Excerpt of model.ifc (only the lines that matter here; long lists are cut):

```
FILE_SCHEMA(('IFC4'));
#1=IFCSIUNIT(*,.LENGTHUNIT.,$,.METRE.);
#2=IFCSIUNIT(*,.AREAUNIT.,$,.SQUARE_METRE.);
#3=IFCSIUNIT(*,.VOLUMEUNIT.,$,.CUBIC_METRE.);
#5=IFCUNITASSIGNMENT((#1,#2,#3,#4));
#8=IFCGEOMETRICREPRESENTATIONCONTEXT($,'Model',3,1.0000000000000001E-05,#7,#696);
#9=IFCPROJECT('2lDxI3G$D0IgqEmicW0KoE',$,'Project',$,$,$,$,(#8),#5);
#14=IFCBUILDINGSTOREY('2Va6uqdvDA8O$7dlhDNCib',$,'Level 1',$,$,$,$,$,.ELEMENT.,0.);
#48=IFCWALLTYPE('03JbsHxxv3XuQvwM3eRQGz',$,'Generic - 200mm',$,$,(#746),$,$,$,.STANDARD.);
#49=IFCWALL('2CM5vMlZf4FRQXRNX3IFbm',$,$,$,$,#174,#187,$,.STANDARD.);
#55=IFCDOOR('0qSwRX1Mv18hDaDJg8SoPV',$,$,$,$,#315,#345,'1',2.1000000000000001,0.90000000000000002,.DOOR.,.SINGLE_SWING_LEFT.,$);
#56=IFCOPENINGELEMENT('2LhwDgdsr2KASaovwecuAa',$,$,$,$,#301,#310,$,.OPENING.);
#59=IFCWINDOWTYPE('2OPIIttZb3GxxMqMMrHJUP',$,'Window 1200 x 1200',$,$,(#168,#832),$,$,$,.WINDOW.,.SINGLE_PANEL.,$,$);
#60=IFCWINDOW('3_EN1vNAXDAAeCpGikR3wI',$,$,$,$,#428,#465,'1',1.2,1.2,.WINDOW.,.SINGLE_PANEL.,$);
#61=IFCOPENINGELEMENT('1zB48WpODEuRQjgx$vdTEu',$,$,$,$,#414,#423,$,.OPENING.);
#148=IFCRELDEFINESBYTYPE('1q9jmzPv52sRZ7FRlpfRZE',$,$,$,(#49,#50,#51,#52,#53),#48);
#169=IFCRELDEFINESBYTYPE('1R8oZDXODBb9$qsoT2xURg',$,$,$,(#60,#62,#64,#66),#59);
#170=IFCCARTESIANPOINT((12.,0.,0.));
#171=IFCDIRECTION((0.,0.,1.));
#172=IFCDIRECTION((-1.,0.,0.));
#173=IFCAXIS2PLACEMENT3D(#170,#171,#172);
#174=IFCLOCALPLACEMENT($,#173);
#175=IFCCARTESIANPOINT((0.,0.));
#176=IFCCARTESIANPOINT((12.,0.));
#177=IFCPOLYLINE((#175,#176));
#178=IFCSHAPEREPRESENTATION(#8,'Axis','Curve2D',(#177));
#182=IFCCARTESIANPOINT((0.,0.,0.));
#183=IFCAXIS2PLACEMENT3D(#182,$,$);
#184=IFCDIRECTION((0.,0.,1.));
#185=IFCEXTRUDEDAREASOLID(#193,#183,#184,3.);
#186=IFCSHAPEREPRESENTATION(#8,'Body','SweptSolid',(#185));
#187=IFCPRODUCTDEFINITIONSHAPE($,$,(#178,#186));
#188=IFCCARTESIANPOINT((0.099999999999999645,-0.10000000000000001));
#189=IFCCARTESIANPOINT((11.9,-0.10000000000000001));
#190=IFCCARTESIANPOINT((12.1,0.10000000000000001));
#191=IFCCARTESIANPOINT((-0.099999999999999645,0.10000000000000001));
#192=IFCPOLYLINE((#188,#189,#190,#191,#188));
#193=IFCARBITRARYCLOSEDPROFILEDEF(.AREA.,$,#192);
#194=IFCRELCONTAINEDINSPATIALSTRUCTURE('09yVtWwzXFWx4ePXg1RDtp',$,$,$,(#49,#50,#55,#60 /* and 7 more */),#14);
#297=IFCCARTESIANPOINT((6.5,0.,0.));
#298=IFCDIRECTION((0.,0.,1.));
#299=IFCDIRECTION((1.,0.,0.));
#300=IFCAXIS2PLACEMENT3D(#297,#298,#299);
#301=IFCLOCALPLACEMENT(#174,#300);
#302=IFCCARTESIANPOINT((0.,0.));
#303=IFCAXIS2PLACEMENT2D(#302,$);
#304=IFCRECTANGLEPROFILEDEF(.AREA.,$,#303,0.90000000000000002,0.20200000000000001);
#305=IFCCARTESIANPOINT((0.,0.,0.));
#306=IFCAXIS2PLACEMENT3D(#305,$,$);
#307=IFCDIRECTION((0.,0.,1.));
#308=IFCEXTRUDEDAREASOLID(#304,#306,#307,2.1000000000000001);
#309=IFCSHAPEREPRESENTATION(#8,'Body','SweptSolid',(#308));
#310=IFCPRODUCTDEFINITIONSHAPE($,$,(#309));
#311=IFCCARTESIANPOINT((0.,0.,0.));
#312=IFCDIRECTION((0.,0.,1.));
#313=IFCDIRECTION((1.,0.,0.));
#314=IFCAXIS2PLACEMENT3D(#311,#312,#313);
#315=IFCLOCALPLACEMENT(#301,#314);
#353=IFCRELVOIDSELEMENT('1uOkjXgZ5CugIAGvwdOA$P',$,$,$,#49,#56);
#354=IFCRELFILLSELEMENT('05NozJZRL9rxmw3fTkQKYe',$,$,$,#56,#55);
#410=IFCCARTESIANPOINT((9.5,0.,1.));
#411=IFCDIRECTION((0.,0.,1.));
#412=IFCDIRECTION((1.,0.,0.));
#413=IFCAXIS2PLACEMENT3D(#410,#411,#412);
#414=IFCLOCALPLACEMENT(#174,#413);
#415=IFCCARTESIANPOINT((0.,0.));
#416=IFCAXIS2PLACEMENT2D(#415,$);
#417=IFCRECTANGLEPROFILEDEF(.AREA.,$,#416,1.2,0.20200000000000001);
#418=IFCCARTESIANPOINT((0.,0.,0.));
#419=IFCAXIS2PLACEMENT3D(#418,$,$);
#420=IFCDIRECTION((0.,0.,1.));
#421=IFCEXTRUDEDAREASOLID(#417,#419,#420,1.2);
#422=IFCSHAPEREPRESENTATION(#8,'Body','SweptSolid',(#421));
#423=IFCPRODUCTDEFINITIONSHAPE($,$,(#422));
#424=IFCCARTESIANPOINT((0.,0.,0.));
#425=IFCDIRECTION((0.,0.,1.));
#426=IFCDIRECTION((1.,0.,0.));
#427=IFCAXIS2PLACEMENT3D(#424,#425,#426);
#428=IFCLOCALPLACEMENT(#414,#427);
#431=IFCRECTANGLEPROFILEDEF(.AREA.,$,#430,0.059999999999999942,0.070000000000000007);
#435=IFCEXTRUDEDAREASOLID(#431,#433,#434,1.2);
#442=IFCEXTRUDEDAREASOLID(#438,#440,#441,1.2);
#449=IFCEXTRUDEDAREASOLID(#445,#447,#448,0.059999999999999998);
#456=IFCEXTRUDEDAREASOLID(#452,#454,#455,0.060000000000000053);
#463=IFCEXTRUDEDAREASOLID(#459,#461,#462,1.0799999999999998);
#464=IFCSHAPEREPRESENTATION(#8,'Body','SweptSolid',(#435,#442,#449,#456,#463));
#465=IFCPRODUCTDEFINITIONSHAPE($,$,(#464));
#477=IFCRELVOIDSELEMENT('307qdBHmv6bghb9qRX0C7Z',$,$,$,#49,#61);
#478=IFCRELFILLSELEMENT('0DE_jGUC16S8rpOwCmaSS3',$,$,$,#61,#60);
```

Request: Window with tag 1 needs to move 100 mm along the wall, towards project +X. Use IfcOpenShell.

```python
import ifcopenshell
import ifcopenshell.api.geometry
import ifcopenshell.util.placement
import ifcopenshell.util.unit

model = ifcopenshell.open("model.ifc")
unit_scale = ifcopenshell.util.unit.calculate_unit_scale(model)

window = model.by_guid("3_EN1vNAXDAAeCpGikR3wI")
opening = window.FillsVoids[0].RelatingOpeningElement
wall = opening.VoidsElements[0].RelatingBuildingElement

wall_matrix = ifcopenshell.util.placement.get_local_placement(wall.ObjectPlacement)
shift = wall_matrix[:3, 0] * -0.1 / unit_scale
before = ifcopenshell.util.placement.get_local_placement(window.ObjectPlacement)[:3, 3].copy()

# The window is placed relative to its opening, so it follows when the opening moves.
matrix = ifcopenshell.util.placement.get_local_placement(opening.ObjectPlacement)
matrix[:3, 3] += shift
ifcopenshell.api.geometry.edit_object_placement(
    model, product=opening, matrix=matrix, is_si=False, should_transform_children=True
)

after = ifcopenshell.util.placement.get_local_placement(window.ObjectPlacement)[:3, 3]
print("window moved by", (after - before).round(3) + 0.0)

model.write("model_edited.ifc")
```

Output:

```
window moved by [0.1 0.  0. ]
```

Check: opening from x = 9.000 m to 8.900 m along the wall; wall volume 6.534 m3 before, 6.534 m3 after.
